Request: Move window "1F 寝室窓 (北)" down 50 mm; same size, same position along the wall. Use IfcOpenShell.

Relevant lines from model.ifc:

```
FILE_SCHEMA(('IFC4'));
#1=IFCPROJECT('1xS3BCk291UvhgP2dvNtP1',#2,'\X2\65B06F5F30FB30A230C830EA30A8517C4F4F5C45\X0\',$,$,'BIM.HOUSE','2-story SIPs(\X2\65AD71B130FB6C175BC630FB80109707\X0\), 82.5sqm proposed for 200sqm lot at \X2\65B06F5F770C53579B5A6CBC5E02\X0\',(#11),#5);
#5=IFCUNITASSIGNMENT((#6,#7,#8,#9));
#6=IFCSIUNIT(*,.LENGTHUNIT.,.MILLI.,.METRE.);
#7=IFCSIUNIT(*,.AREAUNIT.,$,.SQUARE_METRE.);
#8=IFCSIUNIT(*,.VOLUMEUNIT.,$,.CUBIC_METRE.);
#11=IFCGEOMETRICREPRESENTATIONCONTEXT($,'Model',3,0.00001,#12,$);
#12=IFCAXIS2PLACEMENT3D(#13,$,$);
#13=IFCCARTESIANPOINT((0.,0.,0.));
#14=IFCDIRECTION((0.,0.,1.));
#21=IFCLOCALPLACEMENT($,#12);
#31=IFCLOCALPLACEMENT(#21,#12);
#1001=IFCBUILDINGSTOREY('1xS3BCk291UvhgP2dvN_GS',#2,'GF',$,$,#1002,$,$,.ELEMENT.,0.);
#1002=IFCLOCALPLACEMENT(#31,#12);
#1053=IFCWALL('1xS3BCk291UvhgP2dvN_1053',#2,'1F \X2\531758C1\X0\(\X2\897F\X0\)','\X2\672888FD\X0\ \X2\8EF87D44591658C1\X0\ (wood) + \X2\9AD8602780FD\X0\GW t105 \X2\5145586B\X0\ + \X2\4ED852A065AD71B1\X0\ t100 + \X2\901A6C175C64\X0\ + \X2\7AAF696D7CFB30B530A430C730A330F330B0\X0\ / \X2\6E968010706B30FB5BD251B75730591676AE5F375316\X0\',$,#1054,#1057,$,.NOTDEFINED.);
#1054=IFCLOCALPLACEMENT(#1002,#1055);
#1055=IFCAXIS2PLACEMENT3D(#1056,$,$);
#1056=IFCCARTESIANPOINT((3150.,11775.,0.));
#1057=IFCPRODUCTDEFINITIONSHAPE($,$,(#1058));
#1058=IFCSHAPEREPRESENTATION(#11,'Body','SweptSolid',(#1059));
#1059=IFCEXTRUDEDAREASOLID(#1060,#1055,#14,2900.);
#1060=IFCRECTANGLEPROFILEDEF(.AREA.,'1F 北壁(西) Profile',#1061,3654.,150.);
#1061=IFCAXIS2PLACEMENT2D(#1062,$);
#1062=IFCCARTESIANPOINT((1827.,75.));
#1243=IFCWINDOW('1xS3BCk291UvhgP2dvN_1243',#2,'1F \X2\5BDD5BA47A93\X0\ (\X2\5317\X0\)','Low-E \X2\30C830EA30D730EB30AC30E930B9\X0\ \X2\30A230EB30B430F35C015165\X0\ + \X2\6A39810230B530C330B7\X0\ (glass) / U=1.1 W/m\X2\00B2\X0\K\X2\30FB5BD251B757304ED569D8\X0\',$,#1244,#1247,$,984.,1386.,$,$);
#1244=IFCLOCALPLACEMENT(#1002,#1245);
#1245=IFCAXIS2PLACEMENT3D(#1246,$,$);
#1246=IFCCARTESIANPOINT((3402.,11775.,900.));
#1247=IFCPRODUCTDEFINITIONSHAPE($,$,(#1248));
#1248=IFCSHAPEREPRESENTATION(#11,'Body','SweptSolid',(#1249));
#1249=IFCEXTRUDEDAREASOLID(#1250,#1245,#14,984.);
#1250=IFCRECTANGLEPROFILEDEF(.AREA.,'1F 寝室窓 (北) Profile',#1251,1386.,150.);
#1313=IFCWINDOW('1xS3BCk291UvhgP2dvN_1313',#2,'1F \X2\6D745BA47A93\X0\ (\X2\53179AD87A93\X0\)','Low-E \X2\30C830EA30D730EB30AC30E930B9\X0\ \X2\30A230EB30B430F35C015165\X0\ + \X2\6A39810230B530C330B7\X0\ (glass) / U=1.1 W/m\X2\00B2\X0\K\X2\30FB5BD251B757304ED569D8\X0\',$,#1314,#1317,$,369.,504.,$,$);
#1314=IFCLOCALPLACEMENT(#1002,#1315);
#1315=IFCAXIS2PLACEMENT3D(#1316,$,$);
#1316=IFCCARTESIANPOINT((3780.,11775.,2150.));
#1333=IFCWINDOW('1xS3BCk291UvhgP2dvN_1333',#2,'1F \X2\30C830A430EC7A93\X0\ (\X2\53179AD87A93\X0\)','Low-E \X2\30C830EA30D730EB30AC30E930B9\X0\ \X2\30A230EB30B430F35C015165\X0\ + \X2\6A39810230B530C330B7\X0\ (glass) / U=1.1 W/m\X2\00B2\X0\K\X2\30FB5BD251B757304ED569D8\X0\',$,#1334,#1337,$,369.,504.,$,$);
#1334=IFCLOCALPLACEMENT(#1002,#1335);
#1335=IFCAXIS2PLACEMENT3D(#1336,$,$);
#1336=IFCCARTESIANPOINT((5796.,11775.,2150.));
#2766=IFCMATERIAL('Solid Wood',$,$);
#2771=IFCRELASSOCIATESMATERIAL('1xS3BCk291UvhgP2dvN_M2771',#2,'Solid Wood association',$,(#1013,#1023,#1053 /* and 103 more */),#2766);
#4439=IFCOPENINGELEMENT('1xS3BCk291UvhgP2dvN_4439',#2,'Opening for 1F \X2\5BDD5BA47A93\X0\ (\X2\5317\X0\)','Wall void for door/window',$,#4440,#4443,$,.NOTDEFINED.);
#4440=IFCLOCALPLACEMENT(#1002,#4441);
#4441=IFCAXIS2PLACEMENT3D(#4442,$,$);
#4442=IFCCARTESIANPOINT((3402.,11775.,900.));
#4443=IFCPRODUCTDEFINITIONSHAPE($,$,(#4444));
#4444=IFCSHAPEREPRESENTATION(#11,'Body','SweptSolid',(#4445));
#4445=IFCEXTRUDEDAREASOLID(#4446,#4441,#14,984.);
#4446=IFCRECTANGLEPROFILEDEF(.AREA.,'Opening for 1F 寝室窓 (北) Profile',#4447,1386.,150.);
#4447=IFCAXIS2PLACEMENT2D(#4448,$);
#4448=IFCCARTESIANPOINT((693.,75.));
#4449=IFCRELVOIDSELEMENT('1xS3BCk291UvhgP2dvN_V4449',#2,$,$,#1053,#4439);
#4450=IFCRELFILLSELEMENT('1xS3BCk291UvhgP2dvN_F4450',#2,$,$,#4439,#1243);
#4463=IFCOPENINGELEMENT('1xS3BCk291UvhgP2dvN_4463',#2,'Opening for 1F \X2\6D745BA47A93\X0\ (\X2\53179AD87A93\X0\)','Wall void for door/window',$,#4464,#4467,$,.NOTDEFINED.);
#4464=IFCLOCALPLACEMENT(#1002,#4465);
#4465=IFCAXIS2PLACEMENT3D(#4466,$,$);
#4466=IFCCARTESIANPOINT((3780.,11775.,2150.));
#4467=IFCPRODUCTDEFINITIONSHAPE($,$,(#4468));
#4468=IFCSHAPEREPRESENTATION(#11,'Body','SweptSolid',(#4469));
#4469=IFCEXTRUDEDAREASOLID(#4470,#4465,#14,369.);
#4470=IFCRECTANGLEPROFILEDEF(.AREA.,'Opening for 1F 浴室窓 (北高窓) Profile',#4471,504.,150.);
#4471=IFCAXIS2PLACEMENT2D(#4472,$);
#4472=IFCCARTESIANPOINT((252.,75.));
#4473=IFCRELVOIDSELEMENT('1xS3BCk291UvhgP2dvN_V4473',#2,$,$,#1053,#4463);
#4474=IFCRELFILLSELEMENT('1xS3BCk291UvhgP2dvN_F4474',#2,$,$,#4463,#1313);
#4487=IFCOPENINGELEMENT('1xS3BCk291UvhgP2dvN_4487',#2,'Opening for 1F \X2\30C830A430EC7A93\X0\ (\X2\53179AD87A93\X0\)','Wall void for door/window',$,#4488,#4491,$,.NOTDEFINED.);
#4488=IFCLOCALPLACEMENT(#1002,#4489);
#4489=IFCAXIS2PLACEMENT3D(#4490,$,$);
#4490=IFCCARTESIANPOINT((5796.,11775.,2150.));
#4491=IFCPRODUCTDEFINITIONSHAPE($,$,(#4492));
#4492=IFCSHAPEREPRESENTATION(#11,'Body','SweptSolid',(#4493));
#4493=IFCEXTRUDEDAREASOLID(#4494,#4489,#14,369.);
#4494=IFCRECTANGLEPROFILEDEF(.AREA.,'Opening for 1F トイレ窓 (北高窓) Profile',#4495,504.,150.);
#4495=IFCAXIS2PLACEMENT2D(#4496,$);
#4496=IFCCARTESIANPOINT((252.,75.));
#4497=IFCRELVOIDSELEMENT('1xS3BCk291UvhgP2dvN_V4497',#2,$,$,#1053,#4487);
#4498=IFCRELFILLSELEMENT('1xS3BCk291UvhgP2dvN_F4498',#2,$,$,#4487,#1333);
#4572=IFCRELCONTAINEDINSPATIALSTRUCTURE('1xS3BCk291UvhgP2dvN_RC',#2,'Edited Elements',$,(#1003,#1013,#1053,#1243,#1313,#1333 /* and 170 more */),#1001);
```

```python
import numpy as np
import ifcopenshell
import ifcopenshell.api.geometry
import ifcopenshell.util.placement
import ifcopenshell.util.unit

model = ifcopenshell.open("model.ifc")
unit_scale = ifcopenshell.util.unit.calculate_unit_scale(model)

window = model.by_guid("1xS3BCk291UvhgP2dvN_1243")
opening = window.FillsVoids[0].RelatingOpeningElement
dz = -0.05 / unit_scale

shift = np.array([0.0, 0.0, dz])
# The window is not placed relative to its opening, so move both.
for product in (opening, window):
    matrix = ifcopenshell.util.placement.get_local_placement(product.ObjectPlacement)
    matrix[:3, 3] += shift
    ifcopenshell.api.geometry.edit_object_placement(model, product=product, matrix=matrix, is_si=False)

print(f"moved by {dz * unit_scale:+.3f} m")

model.write("model_rev.ifc")
```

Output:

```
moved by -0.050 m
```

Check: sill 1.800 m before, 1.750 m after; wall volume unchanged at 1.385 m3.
